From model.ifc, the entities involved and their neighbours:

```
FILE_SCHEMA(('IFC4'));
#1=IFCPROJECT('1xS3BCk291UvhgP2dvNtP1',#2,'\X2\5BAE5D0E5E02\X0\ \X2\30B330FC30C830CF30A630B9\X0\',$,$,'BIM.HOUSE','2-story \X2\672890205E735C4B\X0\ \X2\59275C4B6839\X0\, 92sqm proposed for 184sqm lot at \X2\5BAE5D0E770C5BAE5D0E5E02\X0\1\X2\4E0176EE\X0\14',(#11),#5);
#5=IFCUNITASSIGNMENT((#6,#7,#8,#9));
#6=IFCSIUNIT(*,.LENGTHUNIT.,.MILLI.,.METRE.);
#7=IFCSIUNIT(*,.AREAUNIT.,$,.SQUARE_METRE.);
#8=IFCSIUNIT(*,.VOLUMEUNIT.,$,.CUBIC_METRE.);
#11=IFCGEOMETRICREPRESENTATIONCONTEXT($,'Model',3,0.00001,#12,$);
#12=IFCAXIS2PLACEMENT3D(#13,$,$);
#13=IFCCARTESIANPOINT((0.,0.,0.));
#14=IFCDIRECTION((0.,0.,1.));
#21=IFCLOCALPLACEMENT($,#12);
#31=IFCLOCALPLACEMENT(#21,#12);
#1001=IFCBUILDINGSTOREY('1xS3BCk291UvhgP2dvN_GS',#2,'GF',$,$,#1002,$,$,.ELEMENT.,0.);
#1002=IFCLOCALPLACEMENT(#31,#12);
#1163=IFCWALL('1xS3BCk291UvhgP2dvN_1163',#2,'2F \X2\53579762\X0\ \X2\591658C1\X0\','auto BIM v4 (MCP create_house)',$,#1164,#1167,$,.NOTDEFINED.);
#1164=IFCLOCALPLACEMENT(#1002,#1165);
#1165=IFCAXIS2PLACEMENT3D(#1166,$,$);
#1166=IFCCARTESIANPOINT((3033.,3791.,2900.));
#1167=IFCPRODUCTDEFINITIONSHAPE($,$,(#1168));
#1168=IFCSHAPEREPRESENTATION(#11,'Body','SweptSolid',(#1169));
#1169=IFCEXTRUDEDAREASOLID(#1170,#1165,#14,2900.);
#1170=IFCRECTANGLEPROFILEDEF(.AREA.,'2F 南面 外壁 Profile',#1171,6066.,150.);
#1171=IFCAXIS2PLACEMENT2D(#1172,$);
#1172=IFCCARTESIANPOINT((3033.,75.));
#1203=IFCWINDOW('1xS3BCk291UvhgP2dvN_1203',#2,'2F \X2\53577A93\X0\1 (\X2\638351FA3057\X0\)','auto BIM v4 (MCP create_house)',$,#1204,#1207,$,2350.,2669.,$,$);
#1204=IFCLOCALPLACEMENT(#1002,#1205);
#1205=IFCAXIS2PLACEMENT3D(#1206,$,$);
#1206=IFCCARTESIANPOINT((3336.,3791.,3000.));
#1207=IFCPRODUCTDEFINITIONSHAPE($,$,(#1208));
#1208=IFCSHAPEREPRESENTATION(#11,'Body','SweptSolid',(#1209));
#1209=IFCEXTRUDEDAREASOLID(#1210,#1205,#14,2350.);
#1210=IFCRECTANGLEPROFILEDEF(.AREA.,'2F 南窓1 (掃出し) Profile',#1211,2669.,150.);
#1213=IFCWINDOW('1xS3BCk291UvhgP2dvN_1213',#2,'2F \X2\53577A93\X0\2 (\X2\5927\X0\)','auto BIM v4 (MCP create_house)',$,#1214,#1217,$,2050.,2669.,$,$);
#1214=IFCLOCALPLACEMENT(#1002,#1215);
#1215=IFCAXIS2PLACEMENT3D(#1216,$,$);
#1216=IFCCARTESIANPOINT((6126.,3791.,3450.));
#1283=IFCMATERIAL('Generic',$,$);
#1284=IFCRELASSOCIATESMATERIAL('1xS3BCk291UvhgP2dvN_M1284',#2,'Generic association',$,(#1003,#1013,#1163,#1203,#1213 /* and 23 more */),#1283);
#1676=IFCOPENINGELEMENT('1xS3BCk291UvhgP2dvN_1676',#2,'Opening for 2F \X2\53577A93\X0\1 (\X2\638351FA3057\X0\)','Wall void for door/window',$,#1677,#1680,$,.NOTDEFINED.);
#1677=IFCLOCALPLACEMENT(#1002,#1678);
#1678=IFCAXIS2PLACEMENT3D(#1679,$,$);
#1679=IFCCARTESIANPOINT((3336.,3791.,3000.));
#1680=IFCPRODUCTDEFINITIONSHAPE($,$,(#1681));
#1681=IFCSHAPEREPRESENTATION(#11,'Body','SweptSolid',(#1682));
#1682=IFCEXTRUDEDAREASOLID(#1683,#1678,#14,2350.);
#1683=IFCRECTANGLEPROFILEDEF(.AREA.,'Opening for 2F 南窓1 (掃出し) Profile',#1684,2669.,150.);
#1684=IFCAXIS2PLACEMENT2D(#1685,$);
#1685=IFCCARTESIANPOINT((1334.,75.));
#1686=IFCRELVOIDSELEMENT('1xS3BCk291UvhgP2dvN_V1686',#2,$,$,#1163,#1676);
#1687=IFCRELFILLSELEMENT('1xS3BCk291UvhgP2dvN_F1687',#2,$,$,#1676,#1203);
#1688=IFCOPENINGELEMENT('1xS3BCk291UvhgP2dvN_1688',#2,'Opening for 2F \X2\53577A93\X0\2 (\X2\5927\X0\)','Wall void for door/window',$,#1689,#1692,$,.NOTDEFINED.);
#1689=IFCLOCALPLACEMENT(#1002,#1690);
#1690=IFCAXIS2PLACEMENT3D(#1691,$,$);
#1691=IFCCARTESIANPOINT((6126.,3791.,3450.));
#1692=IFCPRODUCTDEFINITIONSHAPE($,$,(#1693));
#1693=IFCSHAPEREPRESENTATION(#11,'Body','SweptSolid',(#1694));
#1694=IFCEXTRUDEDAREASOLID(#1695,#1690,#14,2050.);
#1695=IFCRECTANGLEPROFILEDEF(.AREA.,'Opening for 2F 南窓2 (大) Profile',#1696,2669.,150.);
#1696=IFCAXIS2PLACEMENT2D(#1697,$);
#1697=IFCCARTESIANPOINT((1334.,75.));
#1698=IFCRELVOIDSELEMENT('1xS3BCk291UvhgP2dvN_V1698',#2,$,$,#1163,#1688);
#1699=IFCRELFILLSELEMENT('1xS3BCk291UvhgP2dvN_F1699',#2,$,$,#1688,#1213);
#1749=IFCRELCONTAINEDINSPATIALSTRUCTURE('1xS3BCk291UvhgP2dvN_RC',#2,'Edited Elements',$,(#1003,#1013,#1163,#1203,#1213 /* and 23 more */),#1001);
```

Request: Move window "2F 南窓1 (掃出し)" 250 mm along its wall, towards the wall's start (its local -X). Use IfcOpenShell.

```python
import ifcopenshell
import ifcopenshell.api.geometry
import ifcopenshell.util.placement
import ifcopenshell.util.unit

model = ifcopenshell.open("model.ifc")
unit_scale = ifcopenshell.util.unit.calculate_unit_scale(model)

window = model.by_guid("1xS3BCk291UvhgP2dvN_1203")
opening = window.FillsVoids[0].RelatingOpeningElement
wall = opening.VoidsElements[0].RelatingBuildingElement

wall_matrix = ifcopenshell.util.placement.get_local_placement(wall.ObjectPlacement)
shift = wall_matrix[:3, 0] * -0.25 / unit_scale
before = ifcopenshell.util.placement.get_local_placement(window.ObjectPlacement)[:3, 3].copy()

# The window is not placed relative to its opening, so move both.
for product in (opening, window):
    matrix = ifcopenshell.util.placement.get_local_placement(product.ObjectPlacement)
    matrix[:3, 3] += shift
    ifcopenshell.api.geometry.edit_object_placement(model, product=product, matrix=matrix, is_si=False)

after = ifcopenshell.util.placement.get_local_placement(window.ObjectPlacement)[:3, 3]
print("window moved by", (after - before).round(3) + 0.0)

model.write("model_edited.ifc")
```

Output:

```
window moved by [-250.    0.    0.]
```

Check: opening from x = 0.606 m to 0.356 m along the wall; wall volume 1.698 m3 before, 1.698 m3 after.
